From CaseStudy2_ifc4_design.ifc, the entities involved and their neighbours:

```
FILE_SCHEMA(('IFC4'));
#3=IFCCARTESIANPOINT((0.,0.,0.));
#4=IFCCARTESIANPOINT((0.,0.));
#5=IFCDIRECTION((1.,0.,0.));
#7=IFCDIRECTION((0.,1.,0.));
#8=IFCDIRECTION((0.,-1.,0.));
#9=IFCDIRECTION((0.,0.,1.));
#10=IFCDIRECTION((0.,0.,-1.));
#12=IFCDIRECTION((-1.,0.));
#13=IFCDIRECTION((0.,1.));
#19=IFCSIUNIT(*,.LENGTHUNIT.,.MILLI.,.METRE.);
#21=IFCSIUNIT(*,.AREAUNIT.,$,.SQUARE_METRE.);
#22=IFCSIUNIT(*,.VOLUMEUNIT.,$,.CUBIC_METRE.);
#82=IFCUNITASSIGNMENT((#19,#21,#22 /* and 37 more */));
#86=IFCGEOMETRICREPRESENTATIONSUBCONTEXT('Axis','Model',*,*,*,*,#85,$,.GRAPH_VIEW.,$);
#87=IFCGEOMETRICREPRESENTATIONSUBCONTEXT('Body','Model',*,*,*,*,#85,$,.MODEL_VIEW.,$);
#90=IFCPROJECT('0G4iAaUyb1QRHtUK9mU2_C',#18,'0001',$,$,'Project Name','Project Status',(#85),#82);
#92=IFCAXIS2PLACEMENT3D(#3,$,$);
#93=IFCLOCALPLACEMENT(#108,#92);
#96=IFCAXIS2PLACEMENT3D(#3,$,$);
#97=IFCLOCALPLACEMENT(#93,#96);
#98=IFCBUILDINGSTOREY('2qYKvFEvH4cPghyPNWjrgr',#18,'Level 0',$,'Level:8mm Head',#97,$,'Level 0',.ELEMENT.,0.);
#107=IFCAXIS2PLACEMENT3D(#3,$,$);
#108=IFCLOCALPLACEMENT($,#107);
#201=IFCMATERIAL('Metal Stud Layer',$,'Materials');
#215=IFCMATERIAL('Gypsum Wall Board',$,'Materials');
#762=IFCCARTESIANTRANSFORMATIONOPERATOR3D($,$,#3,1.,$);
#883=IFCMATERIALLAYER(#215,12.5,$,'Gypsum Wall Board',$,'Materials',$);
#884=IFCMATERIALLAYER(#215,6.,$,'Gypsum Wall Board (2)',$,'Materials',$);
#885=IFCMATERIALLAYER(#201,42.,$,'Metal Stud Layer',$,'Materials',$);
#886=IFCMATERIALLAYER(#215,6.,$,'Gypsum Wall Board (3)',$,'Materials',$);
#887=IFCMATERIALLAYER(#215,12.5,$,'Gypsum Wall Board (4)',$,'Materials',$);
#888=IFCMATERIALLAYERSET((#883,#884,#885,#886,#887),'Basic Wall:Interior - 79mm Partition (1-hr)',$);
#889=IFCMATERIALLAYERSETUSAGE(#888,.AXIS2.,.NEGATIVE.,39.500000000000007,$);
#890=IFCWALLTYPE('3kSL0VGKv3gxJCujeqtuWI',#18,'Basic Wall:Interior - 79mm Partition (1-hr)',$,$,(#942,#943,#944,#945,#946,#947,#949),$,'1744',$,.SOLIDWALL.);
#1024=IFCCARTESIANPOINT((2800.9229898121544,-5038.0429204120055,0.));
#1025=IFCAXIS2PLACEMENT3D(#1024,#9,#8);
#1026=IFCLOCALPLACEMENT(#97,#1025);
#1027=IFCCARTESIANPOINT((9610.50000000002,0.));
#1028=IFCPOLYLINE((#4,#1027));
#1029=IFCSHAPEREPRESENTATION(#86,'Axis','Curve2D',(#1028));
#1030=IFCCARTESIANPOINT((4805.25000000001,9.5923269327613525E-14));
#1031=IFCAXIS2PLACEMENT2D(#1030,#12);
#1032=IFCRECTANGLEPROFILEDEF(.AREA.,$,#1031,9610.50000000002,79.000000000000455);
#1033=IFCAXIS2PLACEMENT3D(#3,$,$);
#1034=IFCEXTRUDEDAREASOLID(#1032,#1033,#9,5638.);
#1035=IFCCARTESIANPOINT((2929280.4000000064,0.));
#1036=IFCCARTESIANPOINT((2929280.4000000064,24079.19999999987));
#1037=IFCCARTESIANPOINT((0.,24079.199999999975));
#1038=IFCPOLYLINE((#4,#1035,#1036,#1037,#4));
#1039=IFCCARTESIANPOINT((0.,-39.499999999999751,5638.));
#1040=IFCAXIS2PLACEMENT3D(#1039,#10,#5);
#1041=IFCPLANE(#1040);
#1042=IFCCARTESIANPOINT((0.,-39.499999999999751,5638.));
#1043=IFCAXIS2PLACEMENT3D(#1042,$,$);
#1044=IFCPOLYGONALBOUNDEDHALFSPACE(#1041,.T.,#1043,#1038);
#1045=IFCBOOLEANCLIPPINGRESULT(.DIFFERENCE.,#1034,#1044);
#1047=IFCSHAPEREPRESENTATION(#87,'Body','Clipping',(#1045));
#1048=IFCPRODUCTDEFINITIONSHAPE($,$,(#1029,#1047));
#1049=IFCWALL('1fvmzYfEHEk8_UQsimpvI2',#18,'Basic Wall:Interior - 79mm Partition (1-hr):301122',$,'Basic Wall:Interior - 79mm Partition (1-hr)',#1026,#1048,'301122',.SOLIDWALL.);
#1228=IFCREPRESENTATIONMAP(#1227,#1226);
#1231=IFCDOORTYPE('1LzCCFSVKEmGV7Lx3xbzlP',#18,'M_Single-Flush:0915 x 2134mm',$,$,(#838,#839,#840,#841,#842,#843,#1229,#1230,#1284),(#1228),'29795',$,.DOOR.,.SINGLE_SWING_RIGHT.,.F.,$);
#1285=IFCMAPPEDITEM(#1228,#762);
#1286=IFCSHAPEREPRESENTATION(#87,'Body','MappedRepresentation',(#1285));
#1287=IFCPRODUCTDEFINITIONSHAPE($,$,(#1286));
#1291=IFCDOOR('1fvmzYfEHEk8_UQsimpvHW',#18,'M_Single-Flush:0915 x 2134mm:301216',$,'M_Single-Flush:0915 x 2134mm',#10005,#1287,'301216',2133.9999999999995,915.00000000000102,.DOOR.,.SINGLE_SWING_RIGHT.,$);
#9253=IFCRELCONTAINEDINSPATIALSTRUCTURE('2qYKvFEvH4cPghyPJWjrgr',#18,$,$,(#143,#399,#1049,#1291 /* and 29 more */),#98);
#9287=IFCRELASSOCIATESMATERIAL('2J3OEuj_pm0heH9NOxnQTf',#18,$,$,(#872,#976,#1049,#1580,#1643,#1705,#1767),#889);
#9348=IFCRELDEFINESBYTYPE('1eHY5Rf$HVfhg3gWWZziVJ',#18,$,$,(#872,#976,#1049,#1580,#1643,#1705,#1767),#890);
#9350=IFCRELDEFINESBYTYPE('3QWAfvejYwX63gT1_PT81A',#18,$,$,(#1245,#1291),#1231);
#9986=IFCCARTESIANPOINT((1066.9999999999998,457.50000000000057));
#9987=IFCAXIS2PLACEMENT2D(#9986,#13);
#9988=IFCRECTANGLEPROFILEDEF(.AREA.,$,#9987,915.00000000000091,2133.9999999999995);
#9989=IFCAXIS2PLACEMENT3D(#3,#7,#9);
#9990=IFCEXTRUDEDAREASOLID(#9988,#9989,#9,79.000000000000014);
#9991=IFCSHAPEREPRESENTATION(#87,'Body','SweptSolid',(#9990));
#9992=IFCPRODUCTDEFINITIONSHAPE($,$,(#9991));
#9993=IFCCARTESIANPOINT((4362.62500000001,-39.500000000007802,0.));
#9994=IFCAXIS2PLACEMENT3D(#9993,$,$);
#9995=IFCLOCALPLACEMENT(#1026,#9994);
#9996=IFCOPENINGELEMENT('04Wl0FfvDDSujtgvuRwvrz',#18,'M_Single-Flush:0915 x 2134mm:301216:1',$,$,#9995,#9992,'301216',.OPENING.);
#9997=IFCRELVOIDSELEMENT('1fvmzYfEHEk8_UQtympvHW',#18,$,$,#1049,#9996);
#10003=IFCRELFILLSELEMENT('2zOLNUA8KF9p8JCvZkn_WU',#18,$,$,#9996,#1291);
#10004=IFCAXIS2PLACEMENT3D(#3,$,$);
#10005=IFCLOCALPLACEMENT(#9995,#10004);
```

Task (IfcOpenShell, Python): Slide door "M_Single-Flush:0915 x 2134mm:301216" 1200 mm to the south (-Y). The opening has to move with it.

```python
import ifcopenshell
import ifcopenshell.api.geometry
import ifcopenshell.util.placement
import ifcopenshell.util.unit

model = ifcopenshell.open("CaseStudy2_ifc4_design.ifc")
unit_scale = ifcopenshell.util.unit.calculate_unit_scale(model)

door = model.by_id(1291)
opening = door.FillsVoids[0].RelatingOpeningElement
wall = opening.VoidsElements[0].RelatingBuildingElement

wall_matrix = ifcopenshell.util.placement.get_local_placement(wall.ObjectPlacement)
shift = wall_matrix[:3, 0] * 1.2 / unit_scale
before = ifcopenshell.util.placement.get_local_placement(door.ObjectPlacement)[:3, 3].copy()

# The door is placed relative to its opening, so it follows when the opening moves.
matrix = ifcopenshell.util.placement.get_local_placement(opening.ObjectPlacement)
matrix[:3, 3] += shift
ifcopenshell.api.geometry.edit_object_placement(
    model, product=opening, matrix=matrix, is_si=False, should_transform_children=True
)

after = ifcopenshell.util.placement.get_local_placement(door.ObjectPlacement)[:3, 3]
print("door moved by", (after - before).round(3) + 0.0)

model.write("CaseStudy2_ifc4_design-out.ifc")
```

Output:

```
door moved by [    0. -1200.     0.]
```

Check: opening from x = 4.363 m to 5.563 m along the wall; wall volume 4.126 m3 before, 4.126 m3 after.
